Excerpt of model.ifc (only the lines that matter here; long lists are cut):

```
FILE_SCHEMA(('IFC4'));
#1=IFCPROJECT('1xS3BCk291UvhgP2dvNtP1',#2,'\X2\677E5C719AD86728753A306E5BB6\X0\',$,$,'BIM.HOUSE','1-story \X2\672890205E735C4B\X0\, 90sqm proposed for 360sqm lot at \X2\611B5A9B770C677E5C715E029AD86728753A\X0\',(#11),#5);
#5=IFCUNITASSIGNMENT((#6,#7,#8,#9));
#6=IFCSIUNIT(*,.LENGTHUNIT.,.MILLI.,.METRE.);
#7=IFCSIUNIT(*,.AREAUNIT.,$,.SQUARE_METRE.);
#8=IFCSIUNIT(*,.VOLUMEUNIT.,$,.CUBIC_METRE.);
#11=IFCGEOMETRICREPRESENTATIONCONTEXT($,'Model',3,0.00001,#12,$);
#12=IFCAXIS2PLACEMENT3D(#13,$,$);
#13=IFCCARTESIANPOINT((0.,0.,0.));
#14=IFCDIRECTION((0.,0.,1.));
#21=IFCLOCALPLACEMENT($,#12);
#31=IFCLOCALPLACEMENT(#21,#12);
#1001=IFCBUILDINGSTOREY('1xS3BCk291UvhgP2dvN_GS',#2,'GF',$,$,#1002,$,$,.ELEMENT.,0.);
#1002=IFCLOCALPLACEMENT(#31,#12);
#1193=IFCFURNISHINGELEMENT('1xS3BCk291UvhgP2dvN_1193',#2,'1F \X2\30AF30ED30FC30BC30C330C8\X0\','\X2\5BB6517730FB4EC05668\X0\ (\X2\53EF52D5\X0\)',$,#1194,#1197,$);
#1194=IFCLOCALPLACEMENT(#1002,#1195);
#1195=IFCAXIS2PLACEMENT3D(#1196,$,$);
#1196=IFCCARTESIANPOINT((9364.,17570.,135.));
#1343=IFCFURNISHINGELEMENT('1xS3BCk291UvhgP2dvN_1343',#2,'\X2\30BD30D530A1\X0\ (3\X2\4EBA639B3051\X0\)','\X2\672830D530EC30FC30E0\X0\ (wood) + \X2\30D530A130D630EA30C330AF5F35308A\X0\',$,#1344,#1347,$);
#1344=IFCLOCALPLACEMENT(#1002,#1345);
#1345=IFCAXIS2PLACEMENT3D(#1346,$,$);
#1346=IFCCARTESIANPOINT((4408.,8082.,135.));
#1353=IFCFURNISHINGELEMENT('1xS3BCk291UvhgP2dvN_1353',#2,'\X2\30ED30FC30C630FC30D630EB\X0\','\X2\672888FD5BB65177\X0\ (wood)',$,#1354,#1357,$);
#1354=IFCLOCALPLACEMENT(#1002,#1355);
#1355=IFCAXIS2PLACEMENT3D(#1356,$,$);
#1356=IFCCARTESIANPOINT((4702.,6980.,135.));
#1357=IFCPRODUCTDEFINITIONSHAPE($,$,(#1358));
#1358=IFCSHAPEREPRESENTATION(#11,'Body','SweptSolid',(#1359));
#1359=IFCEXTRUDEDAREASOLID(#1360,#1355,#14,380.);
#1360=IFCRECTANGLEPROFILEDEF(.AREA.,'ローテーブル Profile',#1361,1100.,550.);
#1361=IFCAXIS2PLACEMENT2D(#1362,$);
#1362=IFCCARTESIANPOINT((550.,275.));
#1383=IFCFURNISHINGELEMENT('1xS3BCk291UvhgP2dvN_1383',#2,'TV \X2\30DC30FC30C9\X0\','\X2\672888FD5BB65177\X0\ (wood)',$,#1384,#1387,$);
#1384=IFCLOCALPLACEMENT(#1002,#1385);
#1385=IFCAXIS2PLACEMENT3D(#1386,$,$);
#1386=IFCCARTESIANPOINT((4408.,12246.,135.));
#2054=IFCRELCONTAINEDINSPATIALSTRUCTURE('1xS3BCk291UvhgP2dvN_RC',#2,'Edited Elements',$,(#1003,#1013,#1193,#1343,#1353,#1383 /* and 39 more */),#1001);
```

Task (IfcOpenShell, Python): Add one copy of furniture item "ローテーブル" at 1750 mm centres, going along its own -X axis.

```python
import ifcopenshell
import ifcopenshell.api.geometry
import ifcopenshell.api.root
import ifcopenshell.util.element
import ifcopenshell.util.placement
import ifcopenshell.util.unit

model = ifcopenshell.open("model.ifc")
unit_scale = ifcopenshell.util.unit.calculate_unit_scale(model)


def reuse_history(source, copy):
    """copy_class also copies each property set's owner history, people and application; keep the originals."""
    for rel in copy.IsDefinedBy:
        if rel.is_a("IfcRelDefinesByProperties") and (history := rel.RelatingPropertyDefinition.OwnerHistory):
            rel.RelatingPropertyDefinition.OwnerHistory = source.OwnerHistory
            ifcopenshell.util.element.remove_deep2(model, history)


source = model.by_guid("1xS3BCk291UvhgP2dvN_1353")
base = ifcopenshell.util.placement.get_local_placement(source.ObjectPlacement)
step = -base[:3, 0] * 1.75 / unit_scale

for i in range(1, 2):
    copy = ifcopenshell.api.root.copy_class(model, product=source)
    copy.Representation = ifcopenshell.util.element.copy_deep(
        model, source.Representation, exclude=["IfcGeometricRepresentationContext", "IfcRepresentationMap"]
    )
    reuse_history(source, copy)
    matrix = base.copy()
    matrix[:3, 3] += i * step
    print("added at", matrix[:3, 3].round(3) + 0.0)
    ifcopenshell.api.geometry.edit_object_placement(model, product=copy, matrix=matrix, is_si=False)

model.write("model-out.ifc")
```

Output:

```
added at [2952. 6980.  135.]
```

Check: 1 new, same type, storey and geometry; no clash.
